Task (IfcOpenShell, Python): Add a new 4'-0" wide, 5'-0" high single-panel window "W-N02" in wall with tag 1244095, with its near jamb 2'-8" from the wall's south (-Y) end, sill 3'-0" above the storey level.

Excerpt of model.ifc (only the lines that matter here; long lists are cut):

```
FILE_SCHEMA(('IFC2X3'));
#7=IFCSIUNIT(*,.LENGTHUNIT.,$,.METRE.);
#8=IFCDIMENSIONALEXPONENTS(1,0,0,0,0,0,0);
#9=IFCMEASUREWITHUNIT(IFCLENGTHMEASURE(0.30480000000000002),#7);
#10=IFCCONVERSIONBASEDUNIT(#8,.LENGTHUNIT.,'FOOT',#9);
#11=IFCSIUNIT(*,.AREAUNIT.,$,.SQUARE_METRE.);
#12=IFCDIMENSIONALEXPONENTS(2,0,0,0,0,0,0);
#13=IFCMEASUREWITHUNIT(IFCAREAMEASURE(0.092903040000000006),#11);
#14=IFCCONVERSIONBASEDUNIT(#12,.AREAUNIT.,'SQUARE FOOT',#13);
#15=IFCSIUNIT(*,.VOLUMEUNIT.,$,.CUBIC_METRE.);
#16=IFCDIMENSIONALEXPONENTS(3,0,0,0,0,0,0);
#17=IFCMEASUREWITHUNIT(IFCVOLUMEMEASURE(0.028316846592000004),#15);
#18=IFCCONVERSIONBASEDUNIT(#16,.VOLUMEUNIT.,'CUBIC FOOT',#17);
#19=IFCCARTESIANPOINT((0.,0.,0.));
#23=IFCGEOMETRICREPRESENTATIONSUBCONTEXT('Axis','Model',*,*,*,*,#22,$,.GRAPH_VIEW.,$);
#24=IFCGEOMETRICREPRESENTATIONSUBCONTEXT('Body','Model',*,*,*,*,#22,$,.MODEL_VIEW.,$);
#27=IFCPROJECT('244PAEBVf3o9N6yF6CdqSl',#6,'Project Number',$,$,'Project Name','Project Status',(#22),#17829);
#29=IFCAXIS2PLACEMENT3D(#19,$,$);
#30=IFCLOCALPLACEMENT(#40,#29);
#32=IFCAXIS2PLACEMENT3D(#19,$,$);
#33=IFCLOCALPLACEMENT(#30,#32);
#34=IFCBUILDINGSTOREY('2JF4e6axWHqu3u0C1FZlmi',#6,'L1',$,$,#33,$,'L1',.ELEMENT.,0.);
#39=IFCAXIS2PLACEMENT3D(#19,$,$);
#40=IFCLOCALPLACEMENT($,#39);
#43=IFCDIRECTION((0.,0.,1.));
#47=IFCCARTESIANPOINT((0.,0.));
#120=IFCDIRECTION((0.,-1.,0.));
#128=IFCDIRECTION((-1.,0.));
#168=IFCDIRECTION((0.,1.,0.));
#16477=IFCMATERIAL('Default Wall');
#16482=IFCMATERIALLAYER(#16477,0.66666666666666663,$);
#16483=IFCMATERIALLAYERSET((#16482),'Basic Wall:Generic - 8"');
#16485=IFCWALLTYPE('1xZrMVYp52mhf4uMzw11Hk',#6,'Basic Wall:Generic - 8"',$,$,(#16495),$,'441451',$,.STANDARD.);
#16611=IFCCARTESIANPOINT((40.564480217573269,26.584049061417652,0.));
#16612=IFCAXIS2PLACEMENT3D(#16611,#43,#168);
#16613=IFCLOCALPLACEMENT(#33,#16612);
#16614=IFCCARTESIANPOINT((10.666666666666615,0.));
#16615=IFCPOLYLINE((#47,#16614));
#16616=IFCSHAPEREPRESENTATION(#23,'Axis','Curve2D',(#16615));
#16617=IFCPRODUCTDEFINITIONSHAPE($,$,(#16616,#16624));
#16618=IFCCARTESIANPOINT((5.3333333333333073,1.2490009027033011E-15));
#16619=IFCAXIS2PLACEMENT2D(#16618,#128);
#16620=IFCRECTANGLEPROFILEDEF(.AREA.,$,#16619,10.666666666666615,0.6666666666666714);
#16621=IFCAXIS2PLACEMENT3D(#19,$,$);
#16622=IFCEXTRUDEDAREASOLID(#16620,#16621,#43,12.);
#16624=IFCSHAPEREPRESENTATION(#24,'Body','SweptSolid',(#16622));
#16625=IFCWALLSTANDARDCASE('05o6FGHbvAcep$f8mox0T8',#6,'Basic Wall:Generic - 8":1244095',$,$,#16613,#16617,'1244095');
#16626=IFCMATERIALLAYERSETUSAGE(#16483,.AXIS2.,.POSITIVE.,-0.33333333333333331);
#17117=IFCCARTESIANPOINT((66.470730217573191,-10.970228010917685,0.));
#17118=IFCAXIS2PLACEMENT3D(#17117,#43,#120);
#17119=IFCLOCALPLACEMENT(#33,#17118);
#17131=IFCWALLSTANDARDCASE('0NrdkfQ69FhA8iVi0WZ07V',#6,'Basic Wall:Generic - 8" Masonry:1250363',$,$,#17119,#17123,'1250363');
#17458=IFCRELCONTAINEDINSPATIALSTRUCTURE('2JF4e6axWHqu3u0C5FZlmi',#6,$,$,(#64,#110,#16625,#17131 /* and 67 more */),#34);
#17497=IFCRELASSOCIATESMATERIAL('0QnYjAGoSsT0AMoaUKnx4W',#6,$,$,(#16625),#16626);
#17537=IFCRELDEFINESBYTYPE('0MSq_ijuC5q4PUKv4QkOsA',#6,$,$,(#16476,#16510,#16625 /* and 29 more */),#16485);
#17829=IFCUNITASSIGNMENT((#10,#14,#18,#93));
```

```python
import numpy as np
import ifcopenshell
import ifcopenshell.api.feature
import ifcopenshell.api.geometry
import ifcopenshell.api.root
import ifcopenshell.api.spatial
import ifcopenshell.api.type
import ifcopenshell.geom
import ifcopenshell.util.element
import ifcopenshell.util.placement
import ifcopenshell.util.representation
import ifcopenshell.util.shape
import ifcopenshell.util.unit

model = ifcopenshell.open("model.ifc")
unit_scale = ifcopenshell.util.unit.calculate_unit_scale(model)
settings = ifcopenshell.geom.settings()


def volume(element):
    """Net volume in cubic metres, openings subtracted."""
    shape = ifcopenshell.geom.create_shape(settings, element)
    return ifcopenshell.util.shape.get_volume(shape.geometry)


wall = model.by_guid("05o6FGHbvAcep$f8mox0T8")
storey = ifcopenshell.util.element.get_container(wall, ifc_class="IfcBuildingStorey")
context = ifcopenshell.util.representation.get_context(model, "Model", "Body", "MODEL_VIEW")
before = volume(wall)

width, height, from_end, sill = 1.2192, 1.524, 0.8128, 0.9144  # metres

# The wall runs along its own X axis, and the end named is its -X end.
wall_shape = ifcopenshell.geom.create_shape(settings, wall)
x, y, z = ifcopenshell.util.shape.get_vertices(wall_shape.geometry).T
start = x.min() + from_end
face, thickness = float(y.min()), float(y.max() - y.min())
wall_matrix = ifcopenshell.util.placement.get_local_placement(wall.ObjectPlacement)
level = ifcopenshell.util.placement.get_local_placement(storey.ObjectPlacement)[2, 3]


def in_wall(x, y):
    """Placement at x, y metres in the wall's axes, at sill height."""
    matrix = wall_matrix.copy()
    matrix[:, 3] = wall_matrix @ np.array([x / unit_scale, y / unit_scale, 0.0, 1.0])
    matrix[2, 3] = level + sill / unit_scale
    return matrix


# Opening: a box that overshoots both wall faces by 50 mm.
opening = ifcopenshell.api.root.create_entity(model, ifc_class="IfcOpeningElement")
box = ifcopenshell.api.geometry.add_wall_representation(
    model, context=context, length=width, height=height, thickness=thickness + 0.1
)
ifcopenshell.api.geometry.assign_representation(model, product=opening, representation=box)
ifcopenshell.api.geometry.edit_object_placement(model, product=opening, matrix=in_wall(start, face - 0.05), is_si=False)
ifcopenshell.api.feature.add_feature(model, feature=opening, element=wall)

window = ifcopenshell.api.root.create_entity(model, ifc_class="IfcWindow", name="W-N02")
window.OverallWidth, window.OverallHeight = width / unit_scale, height / unit_scale
body = ifcopenshell.api.geometry.add_window_representation(
    model,
    context=context,
    overall_width=window.OverallWidth,
    overall_height=window.OverallHeight,
    partition_type="SINGLE_PANEL",
)
ifcopenshell.api.geometry.assign_representation(model, product=window, representation=body)
ifcopenshell.api.spatial.assign_container(model, products=[window], relating_structure=storey)
fills = ifcopenshell.api.feature.add_filling(model, opening=opening, element=window)
fills.OwnerHistory = window.OwnerHistory  # required in IFC2X3

# IFC2X3 keeps the operation on the window style.
style = ifcopenshell.api.root.create_entity(model, ifc_class="IfcWindowStyle", name="W-N02")
style.OperationType, style.ConstructionType = "SINGLE_PANEL", "NOTDEFINED"
style.ParameterTakesPrecedence = style.Sizeable = False
ifcopenshell.api.type.assign_type(model, related_objects=[window], relating_type=style)

# Centre the window in the wall's thickness.
ifcopenshell.api.geometry.edit_object_placement(model, product=window, matrix=in_wall(start, face), is_si=False)
window_shape = ifcopenshell.geom.create_shape(settings, window)
depth = ifcopenshell.util.shape.get_vertices(window_shape.geometry)[:, 1]
offset = face + thickness / 2 - (depth.min() + depth.max()) / 2
ifcopenshell.api.geometry.edit_object_placement(model, product=window, matrix=in_wall(start, offset), is_si=False)

after = volume(wall)

print(f"wall volume {before:.3f} -> {after:.3f} m3")

model.write("model-out.ifc")
```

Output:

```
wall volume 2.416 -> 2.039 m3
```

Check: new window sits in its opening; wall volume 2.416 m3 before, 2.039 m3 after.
